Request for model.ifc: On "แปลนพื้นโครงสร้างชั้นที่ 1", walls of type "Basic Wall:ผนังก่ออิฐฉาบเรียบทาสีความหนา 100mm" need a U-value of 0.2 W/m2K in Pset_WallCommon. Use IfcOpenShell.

First a look at what the model holds.

```python
import ifcopenshell
import ifcopenshell.util.element

model = ifcopenshell.open("model.ifc")
print(model.schema)
storey = next(s for s in model.by_type("IfcBuildingStorey") if s.Name == "แปลนพื้นโครงสร้างชั้นที่ 1")
walls = [e for e in ifcopenshell.util.element.get_decomposition(storey) if e.is_a("IfcWall")]
seen = {}
for e in walls:
    element_type = ifcopenshell.util.element.get_type(e)
    key = (element_type.Name if element_type != e and element_type else None, ifcopenshell.util.element.get_pset(e, "Pset_WallCommon", "ThermalTransmittance"))
    seen[key] = seen.get(key, 0) + 1
for (name, value), count in sorted(seen.items(), key=str):
    print(count, "x", name, "|", value)
```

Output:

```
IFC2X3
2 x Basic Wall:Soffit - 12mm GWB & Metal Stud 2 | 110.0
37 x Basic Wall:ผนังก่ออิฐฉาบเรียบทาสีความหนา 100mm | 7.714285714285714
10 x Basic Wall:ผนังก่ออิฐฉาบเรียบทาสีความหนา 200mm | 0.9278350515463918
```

```python
import ifcopenshell
import ifcopenshell.api.pset
import ifcopenshell.util.element

model = ifcopenshell.open("model.ifc")

storey = next(s for s in model.by_type("IfcBuildingStorey") if s.Name == "แปลนพื้นโครงสร้างชั้นที่ 1")
walls = [e for e in ifcopenshell.util.element.get_decomposition(storey) if e.is_a("IfcWall")]

count = 0
for e in walls:
    element_type = ifcopenshell.util.element.get_type(e)
    if element_type in (None, e) or element_type.Name != "Basic Wall:ผนังก่ออิฐฉาบเรียบทาสีความหนา 100mm":
        continue
    # add_pset returns the element's existing set when there is one.
    pset = ifcopenshell.api.pset.add_pset(model, product=e, name="Pset_WallCommon")
    ifcopenshell.api.pset.edit_pset(model, pset=pset, properties={"ThermalTransmittance": 0.2})
    count += 1

print(count, "walls updated")

model.write("model_v2.ifc")
```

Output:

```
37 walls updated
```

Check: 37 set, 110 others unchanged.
